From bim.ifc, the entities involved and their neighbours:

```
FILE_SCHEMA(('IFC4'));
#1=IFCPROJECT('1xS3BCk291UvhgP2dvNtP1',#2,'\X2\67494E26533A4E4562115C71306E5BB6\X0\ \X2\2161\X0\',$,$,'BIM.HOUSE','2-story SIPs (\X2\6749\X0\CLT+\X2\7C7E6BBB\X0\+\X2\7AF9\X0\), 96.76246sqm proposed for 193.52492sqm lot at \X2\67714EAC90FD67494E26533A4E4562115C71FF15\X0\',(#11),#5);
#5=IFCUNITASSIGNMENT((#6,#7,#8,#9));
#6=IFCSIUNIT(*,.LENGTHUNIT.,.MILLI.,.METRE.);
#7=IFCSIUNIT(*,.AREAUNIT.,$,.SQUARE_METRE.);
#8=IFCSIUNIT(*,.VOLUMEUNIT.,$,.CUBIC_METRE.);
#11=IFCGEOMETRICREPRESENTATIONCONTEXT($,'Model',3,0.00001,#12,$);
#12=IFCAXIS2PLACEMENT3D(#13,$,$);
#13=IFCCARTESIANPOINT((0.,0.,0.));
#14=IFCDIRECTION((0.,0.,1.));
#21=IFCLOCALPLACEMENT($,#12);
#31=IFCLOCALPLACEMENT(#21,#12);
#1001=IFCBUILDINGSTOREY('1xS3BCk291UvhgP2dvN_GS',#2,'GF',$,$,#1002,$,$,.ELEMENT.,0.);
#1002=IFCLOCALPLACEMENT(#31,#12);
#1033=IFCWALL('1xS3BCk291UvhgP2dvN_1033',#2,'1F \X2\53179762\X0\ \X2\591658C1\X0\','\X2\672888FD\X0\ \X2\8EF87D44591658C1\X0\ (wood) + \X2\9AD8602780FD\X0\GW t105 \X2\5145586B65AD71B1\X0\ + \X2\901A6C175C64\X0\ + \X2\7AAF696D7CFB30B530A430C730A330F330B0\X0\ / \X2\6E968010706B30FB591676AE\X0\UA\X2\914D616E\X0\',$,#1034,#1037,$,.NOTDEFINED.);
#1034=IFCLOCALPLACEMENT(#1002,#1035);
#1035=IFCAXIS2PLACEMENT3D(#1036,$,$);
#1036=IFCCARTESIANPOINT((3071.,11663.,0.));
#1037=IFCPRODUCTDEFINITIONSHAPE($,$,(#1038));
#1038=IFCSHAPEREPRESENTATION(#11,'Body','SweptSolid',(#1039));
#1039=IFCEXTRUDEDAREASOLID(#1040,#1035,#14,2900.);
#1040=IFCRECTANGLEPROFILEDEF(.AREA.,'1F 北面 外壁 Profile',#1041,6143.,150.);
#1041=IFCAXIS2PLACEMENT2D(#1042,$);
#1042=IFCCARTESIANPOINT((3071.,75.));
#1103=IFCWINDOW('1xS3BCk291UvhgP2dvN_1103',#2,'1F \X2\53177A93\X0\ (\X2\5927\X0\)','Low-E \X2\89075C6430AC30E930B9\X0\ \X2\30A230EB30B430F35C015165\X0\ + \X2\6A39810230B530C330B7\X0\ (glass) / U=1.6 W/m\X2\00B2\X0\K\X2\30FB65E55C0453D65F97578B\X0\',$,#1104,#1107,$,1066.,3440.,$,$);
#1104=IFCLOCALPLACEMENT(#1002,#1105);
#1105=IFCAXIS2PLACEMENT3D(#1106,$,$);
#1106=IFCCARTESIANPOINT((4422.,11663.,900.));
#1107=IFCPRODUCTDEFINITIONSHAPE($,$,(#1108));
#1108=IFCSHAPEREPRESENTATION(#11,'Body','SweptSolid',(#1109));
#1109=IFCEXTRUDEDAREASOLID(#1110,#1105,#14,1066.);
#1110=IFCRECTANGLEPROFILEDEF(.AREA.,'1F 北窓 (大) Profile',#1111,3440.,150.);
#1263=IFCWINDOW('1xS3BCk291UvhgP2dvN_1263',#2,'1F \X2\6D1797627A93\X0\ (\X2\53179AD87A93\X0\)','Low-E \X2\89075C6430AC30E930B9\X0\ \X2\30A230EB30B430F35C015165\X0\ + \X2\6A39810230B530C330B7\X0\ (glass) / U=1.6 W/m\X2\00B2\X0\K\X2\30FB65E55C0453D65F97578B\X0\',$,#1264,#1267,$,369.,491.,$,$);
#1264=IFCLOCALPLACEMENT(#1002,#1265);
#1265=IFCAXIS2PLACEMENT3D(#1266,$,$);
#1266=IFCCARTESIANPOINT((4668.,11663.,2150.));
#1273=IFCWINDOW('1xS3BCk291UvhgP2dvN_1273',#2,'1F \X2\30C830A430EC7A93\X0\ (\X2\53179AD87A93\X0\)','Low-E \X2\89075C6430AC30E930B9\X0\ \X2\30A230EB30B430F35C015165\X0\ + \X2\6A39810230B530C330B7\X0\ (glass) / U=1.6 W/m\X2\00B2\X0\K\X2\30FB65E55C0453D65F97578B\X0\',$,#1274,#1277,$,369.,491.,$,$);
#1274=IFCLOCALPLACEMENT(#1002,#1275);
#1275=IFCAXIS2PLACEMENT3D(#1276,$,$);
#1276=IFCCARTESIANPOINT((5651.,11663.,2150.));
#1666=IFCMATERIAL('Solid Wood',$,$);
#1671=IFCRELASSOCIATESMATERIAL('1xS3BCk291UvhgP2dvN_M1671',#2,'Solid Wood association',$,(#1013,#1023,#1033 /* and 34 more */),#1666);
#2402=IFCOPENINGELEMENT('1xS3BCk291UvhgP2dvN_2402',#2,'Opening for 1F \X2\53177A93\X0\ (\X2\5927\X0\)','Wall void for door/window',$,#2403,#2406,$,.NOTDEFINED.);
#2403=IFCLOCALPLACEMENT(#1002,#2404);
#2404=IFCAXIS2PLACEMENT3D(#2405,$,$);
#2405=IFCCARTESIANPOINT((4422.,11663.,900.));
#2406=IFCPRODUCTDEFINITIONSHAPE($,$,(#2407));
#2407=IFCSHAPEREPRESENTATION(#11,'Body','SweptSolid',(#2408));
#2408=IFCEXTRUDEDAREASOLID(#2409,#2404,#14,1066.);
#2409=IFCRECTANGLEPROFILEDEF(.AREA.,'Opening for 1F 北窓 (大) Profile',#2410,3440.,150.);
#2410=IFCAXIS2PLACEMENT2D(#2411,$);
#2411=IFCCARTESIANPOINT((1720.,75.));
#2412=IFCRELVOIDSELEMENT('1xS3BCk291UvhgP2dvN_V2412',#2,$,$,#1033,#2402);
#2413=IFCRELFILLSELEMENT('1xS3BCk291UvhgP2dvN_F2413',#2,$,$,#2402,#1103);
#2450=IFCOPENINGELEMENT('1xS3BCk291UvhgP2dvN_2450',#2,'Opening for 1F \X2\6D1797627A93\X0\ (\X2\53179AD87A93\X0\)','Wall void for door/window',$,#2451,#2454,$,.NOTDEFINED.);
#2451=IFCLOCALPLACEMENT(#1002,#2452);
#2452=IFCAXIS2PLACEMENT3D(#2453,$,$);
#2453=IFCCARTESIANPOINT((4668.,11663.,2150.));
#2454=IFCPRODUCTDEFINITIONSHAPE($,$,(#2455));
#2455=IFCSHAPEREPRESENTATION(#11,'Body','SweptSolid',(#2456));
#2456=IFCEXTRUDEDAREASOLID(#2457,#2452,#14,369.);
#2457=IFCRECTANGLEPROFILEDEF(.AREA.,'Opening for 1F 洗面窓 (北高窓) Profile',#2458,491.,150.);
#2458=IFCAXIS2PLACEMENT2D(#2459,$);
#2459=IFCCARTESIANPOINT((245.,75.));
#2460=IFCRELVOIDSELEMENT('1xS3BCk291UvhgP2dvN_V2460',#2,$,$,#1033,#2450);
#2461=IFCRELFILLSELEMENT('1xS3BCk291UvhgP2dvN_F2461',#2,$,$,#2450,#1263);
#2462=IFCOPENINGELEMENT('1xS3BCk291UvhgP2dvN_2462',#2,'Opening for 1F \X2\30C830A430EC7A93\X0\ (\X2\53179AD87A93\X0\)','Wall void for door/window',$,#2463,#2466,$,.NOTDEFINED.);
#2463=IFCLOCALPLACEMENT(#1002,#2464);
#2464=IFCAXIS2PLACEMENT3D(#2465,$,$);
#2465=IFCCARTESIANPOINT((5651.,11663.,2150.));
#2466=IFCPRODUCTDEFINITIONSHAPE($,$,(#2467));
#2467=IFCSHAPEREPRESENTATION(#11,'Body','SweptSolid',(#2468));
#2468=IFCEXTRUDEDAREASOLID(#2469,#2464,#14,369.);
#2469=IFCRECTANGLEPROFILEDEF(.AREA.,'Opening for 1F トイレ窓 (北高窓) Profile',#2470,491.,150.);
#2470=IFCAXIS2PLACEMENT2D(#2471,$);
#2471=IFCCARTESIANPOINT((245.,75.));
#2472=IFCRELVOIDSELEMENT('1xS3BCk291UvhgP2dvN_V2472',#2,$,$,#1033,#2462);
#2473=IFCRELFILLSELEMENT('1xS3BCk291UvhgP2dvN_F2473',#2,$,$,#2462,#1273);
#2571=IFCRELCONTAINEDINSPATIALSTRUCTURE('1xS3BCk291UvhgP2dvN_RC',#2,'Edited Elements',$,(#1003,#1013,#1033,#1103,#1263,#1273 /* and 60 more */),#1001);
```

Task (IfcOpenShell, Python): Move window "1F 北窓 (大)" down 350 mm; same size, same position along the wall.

```python
import numpy as np
import ifcopenshell
import ifcopenshell.api.geometry
import ifcopenshell.util.placement
import ifcopenshell.util.unit

model = ifcopenshell.open("bim.ifc")
unit_scale = ifcopenshell.util.unit.calculate_unit_scale(model)

window = model.by_guid("1xS3BCk291UvhgP2dvN_1103")
opening = window.FillsVoids[0].RelatingOpeningElement
dz = -0.35 / unit_scale

shift = np.array([0.0, 0.0, dz])
# The window is not placed relative to its opening, so move both.
for product in (opening, window):
    matrix = ifcopenshell.util.placement.get_local_placement(product.ObjectPlacement)
    matrix[:3, 3] += shift
    ifcopenshell.api.geometry.edit_object_placement(model, product=product, matrix=matrix, is_si=False)

print(f"moved by {dz * unit_scale:+.3f} m")

model.write("bim_v2.ifc")
```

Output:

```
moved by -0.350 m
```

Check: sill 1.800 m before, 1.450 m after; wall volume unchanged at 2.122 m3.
